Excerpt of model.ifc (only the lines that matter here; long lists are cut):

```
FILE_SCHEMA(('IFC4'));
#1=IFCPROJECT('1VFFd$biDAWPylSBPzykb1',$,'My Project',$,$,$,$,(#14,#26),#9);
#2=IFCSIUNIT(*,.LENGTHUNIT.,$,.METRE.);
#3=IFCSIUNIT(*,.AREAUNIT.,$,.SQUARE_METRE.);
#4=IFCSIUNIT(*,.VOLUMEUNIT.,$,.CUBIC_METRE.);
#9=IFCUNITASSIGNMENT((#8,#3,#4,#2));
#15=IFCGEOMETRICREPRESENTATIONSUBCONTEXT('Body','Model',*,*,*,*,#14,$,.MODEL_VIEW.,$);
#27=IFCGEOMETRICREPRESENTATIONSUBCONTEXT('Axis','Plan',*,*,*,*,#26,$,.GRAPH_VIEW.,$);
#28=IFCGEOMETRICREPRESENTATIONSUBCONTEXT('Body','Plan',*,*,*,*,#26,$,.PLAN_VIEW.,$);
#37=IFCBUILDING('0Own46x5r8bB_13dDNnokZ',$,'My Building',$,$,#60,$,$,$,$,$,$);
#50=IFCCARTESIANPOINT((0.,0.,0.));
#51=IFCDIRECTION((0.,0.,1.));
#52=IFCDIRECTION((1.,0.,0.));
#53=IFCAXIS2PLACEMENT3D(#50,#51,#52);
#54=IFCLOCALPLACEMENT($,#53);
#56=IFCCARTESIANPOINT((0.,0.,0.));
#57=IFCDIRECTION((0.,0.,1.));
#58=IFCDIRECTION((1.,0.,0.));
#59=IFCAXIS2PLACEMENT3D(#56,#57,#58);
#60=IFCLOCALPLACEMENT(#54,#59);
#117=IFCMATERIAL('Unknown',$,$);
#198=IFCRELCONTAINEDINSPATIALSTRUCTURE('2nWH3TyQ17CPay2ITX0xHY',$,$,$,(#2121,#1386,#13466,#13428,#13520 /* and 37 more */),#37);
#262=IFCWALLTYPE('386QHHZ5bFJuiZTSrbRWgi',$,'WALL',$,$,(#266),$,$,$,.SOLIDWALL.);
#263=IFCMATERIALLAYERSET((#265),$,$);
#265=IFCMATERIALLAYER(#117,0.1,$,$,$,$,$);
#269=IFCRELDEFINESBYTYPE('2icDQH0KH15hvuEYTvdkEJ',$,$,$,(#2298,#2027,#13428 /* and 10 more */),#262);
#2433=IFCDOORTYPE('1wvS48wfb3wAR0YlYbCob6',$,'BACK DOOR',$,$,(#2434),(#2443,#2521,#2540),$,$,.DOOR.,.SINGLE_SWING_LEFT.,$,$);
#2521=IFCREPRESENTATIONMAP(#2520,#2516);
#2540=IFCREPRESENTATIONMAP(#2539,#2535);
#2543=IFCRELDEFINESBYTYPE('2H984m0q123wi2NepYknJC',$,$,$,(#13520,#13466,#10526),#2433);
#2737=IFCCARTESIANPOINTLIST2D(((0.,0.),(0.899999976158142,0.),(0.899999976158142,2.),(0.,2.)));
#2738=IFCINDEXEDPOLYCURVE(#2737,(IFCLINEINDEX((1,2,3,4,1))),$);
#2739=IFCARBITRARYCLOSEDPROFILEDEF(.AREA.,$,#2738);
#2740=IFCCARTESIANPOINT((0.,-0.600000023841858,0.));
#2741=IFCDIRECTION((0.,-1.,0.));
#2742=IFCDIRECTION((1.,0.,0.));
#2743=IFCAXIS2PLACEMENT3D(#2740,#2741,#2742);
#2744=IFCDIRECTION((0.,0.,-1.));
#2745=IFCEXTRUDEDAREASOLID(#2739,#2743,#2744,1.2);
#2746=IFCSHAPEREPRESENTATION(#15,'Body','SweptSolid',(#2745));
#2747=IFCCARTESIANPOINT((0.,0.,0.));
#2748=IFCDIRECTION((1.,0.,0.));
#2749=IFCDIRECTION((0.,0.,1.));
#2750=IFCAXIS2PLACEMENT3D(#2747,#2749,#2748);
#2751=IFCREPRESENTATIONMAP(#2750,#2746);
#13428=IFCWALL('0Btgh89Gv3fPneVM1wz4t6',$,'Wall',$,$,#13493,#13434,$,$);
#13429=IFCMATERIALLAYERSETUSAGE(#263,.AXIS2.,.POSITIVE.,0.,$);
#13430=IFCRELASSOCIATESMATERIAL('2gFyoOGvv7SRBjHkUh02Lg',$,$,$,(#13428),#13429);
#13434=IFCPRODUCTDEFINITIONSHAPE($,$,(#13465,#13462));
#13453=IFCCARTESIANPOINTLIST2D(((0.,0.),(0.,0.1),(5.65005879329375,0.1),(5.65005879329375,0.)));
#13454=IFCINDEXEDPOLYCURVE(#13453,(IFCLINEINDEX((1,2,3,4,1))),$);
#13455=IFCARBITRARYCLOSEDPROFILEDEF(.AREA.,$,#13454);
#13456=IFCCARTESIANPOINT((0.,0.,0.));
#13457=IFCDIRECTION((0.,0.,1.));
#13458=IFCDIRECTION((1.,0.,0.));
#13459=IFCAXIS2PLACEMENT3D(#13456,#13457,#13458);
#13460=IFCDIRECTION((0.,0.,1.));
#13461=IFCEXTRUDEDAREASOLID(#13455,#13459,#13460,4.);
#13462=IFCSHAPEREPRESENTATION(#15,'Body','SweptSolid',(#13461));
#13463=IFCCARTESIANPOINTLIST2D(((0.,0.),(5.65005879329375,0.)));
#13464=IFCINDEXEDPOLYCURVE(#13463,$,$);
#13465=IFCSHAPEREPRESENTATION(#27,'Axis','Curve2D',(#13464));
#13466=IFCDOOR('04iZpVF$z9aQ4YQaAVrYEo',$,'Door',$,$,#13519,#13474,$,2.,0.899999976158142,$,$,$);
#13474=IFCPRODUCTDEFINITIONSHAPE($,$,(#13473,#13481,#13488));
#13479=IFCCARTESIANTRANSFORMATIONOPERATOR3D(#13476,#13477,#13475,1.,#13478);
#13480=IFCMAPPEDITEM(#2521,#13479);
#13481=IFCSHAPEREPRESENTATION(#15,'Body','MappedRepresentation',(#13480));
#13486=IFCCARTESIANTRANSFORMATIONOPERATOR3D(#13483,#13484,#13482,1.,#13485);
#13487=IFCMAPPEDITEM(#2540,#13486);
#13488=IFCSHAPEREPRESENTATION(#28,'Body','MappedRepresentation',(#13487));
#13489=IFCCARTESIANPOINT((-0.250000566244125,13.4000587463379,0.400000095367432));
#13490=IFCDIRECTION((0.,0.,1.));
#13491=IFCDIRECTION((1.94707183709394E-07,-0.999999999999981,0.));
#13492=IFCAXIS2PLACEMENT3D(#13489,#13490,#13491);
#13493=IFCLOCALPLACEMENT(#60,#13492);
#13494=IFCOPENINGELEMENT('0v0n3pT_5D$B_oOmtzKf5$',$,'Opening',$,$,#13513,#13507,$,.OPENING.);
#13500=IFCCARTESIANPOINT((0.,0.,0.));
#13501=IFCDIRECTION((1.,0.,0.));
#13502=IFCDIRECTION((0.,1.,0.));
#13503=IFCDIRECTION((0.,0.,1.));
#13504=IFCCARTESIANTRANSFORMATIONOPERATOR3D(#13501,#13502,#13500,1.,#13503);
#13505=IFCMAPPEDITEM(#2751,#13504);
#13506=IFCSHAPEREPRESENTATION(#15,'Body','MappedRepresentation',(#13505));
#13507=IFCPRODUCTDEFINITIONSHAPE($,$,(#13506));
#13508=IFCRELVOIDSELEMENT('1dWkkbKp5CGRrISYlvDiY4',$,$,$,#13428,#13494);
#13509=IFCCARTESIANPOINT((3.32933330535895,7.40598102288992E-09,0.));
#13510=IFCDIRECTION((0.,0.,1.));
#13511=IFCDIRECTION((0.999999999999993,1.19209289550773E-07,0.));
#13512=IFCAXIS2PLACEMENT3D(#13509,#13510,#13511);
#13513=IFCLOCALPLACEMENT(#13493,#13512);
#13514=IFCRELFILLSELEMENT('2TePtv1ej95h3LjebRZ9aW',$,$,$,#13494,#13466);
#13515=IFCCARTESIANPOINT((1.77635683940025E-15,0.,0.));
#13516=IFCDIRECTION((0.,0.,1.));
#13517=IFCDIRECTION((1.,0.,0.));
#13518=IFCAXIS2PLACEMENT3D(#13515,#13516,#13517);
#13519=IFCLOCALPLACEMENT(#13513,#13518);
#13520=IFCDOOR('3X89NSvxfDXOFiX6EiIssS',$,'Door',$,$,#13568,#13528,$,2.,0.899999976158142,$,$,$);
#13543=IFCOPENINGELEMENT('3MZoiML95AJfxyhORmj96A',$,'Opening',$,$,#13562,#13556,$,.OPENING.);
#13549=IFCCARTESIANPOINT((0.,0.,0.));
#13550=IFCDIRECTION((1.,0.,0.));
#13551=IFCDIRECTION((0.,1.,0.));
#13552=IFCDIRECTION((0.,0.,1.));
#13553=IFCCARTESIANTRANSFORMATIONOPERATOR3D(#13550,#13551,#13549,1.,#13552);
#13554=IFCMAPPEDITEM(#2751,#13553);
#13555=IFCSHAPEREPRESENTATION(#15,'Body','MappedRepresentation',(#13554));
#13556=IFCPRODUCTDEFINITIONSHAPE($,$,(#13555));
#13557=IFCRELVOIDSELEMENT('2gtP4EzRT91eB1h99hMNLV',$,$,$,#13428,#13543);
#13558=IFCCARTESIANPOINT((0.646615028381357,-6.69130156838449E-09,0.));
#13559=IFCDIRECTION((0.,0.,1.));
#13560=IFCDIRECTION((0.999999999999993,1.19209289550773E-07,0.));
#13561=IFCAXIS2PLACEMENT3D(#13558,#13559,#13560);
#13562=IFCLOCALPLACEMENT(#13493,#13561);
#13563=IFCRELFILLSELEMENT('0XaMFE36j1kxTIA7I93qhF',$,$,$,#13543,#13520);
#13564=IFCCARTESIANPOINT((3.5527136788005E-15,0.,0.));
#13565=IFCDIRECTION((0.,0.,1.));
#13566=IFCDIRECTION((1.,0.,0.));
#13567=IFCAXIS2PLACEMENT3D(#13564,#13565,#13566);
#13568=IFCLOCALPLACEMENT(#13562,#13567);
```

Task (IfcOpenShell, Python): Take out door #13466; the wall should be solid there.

```python
import ifcopenshell
import ifcopenshell.api.feature
import ifcopenshell.api.root
import ifcopenshell.geom
import ifcopenshell.util.shape

model = ifcopenshell.open("model.ifc")
settings = ifcopenshell.geom.settings()


def volume(element):
    """Net volume in cubic metres, openings subtracted."""
    shape = ifcopenshell.geom.create_shape(settings, element)
    return ifcopenshell.util.shape.get_volume(shape.geometry)


door = model.by_guid("04iZpVF$z9aQ4YQaAVrYEo")
opening = door.FillsVoids[0].RelatingOpeningElement
wall = opening.VoidsElements[0].RelatingBuildingElement
before = volume(wall)

ifcopenshell.api.root.remove_product(model, product=door)
ifcopenshell.api.feature.remove_feature(model, feature=opening)

after = volume(wall)

print(f"wall volume {before:.3f} -> {after:.3f} m3")

model.write("model_v2.ifc")
```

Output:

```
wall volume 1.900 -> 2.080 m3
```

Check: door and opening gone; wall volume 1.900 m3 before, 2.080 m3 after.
